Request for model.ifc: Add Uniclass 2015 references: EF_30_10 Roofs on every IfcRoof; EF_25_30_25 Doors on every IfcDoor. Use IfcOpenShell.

First a look at what the model holds.

```python
import ifcopenshell

model = ifcopenshell.open("model.ifc")
print(model.schema)
print("classifications:", [c.Name for c in model.by_type("IfcClassification")])
for ifc_class in ("IfcDoor", "IfcRoof", "IfcStair", "IfcWall", "IfcWindow"):
    print(ifc_class, len(model.by_type(ifc_class)))
```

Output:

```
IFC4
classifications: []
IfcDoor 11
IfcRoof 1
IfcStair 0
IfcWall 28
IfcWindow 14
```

```python
import ifcopenshell
import ifcopenshell.api.classification

model = ifcopenshell.open("model.ifc")

system = ifcopenshell.api.classification.add_classification(model, classification="Uniclass 2015")

codes = {
    "IfcRoof": ("EF_30_10", "Roofs"),
    "IfcDoor": ("EF_25_30_25", "Doors"),
}
for ifc_class, (code, name) in codes.items():
    products = model.by_type(ifc_class)
    ifcopenshell.api.classification.add_reference(
        model, products=products, classification=system, identification=code, name=name
    )
    print(code, len(products))

model.write("model_rev.ifc")
```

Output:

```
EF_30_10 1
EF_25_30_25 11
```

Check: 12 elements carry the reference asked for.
